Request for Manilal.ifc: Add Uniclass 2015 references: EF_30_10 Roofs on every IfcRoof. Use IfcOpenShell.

First a look at what the model holds.

```python
import ifcopenshell

model = ifcopenshell.open("Manilal.ifc")
print(model.schema)
print("classifications:", [c.Name for c in model.by_type("IfcClassification")])
for ifc_class in ("IfcDoor", "IfcRoof", "IfcStair", "IfcWall", "IfcWindow"):
    print(ifc_class, len(model.by_type(ifc_class)))
```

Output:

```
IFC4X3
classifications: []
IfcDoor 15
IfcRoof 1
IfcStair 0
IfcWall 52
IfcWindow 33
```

```python
import ifcopenshell
import ifcopenshell.api.classification

model = ifcopenshell.open("Manilal.ifc")

system = ifcopenshell.api.classification.add_classification(model, classification="Uniclass 2015")

codes = {
    "IfcRoof": ("EF_30_10", "Roofs"),
}
for ifc_class, (code, name) in codes.items():
    products = model.by_type(ifc_class)
    ifcopenshell.api.classification.add_reference(
        model, products=products, classification=system, identification=code, name=name
    )
    print(code, len(products))

model.write("Manilal_v2.ifc")
```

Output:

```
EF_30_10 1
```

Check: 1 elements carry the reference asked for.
